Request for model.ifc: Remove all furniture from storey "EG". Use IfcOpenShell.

First a look at what the model holds.

```python
import ifcopenshell
import ifcopenshell.util.element

model = ifcopenshell.open("model.ifc")
print(model.schema)
storey = next(s for s in model.by_type("IfcBuildingStorey") if s.Name == "EG")
furniture = [e for e in ifcopenshell.util.element.get_decomposition(storey) if e.is_a("IfcFurnishingElement")]
seen = {}
for e in furniture:
    element_type = ifcopenshell.util.element.get_type(e)
    name = element_type.Name if element_type not in (None, e) else None
    seen[name] = seen.get(name, 0) + 1
for name, count in sorted(seen.items(), key=str):
    print(count, "x", name)
```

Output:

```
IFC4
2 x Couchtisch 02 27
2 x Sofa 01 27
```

```python
import ifcopenshell
import ifcopenshell.api.root
import ifcopenshell.util.element

model = ifcopenshell.open("model.ifc")

storey = next(s for s in model.by_type("IfcBuildingStorey") if s.Name == "EG")
furniture = [e for e in ifcopenshell.util.element.get_decomposition(storey) if e.is_a("IfcFurnishingElement")]

for e in furniture:
    ifcopenshell.api.root.remove_product(model, product=e)
print(len(furniture), "removed")

model.write("model-out.ifc")
```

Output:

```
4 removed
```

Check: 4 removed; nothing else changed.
